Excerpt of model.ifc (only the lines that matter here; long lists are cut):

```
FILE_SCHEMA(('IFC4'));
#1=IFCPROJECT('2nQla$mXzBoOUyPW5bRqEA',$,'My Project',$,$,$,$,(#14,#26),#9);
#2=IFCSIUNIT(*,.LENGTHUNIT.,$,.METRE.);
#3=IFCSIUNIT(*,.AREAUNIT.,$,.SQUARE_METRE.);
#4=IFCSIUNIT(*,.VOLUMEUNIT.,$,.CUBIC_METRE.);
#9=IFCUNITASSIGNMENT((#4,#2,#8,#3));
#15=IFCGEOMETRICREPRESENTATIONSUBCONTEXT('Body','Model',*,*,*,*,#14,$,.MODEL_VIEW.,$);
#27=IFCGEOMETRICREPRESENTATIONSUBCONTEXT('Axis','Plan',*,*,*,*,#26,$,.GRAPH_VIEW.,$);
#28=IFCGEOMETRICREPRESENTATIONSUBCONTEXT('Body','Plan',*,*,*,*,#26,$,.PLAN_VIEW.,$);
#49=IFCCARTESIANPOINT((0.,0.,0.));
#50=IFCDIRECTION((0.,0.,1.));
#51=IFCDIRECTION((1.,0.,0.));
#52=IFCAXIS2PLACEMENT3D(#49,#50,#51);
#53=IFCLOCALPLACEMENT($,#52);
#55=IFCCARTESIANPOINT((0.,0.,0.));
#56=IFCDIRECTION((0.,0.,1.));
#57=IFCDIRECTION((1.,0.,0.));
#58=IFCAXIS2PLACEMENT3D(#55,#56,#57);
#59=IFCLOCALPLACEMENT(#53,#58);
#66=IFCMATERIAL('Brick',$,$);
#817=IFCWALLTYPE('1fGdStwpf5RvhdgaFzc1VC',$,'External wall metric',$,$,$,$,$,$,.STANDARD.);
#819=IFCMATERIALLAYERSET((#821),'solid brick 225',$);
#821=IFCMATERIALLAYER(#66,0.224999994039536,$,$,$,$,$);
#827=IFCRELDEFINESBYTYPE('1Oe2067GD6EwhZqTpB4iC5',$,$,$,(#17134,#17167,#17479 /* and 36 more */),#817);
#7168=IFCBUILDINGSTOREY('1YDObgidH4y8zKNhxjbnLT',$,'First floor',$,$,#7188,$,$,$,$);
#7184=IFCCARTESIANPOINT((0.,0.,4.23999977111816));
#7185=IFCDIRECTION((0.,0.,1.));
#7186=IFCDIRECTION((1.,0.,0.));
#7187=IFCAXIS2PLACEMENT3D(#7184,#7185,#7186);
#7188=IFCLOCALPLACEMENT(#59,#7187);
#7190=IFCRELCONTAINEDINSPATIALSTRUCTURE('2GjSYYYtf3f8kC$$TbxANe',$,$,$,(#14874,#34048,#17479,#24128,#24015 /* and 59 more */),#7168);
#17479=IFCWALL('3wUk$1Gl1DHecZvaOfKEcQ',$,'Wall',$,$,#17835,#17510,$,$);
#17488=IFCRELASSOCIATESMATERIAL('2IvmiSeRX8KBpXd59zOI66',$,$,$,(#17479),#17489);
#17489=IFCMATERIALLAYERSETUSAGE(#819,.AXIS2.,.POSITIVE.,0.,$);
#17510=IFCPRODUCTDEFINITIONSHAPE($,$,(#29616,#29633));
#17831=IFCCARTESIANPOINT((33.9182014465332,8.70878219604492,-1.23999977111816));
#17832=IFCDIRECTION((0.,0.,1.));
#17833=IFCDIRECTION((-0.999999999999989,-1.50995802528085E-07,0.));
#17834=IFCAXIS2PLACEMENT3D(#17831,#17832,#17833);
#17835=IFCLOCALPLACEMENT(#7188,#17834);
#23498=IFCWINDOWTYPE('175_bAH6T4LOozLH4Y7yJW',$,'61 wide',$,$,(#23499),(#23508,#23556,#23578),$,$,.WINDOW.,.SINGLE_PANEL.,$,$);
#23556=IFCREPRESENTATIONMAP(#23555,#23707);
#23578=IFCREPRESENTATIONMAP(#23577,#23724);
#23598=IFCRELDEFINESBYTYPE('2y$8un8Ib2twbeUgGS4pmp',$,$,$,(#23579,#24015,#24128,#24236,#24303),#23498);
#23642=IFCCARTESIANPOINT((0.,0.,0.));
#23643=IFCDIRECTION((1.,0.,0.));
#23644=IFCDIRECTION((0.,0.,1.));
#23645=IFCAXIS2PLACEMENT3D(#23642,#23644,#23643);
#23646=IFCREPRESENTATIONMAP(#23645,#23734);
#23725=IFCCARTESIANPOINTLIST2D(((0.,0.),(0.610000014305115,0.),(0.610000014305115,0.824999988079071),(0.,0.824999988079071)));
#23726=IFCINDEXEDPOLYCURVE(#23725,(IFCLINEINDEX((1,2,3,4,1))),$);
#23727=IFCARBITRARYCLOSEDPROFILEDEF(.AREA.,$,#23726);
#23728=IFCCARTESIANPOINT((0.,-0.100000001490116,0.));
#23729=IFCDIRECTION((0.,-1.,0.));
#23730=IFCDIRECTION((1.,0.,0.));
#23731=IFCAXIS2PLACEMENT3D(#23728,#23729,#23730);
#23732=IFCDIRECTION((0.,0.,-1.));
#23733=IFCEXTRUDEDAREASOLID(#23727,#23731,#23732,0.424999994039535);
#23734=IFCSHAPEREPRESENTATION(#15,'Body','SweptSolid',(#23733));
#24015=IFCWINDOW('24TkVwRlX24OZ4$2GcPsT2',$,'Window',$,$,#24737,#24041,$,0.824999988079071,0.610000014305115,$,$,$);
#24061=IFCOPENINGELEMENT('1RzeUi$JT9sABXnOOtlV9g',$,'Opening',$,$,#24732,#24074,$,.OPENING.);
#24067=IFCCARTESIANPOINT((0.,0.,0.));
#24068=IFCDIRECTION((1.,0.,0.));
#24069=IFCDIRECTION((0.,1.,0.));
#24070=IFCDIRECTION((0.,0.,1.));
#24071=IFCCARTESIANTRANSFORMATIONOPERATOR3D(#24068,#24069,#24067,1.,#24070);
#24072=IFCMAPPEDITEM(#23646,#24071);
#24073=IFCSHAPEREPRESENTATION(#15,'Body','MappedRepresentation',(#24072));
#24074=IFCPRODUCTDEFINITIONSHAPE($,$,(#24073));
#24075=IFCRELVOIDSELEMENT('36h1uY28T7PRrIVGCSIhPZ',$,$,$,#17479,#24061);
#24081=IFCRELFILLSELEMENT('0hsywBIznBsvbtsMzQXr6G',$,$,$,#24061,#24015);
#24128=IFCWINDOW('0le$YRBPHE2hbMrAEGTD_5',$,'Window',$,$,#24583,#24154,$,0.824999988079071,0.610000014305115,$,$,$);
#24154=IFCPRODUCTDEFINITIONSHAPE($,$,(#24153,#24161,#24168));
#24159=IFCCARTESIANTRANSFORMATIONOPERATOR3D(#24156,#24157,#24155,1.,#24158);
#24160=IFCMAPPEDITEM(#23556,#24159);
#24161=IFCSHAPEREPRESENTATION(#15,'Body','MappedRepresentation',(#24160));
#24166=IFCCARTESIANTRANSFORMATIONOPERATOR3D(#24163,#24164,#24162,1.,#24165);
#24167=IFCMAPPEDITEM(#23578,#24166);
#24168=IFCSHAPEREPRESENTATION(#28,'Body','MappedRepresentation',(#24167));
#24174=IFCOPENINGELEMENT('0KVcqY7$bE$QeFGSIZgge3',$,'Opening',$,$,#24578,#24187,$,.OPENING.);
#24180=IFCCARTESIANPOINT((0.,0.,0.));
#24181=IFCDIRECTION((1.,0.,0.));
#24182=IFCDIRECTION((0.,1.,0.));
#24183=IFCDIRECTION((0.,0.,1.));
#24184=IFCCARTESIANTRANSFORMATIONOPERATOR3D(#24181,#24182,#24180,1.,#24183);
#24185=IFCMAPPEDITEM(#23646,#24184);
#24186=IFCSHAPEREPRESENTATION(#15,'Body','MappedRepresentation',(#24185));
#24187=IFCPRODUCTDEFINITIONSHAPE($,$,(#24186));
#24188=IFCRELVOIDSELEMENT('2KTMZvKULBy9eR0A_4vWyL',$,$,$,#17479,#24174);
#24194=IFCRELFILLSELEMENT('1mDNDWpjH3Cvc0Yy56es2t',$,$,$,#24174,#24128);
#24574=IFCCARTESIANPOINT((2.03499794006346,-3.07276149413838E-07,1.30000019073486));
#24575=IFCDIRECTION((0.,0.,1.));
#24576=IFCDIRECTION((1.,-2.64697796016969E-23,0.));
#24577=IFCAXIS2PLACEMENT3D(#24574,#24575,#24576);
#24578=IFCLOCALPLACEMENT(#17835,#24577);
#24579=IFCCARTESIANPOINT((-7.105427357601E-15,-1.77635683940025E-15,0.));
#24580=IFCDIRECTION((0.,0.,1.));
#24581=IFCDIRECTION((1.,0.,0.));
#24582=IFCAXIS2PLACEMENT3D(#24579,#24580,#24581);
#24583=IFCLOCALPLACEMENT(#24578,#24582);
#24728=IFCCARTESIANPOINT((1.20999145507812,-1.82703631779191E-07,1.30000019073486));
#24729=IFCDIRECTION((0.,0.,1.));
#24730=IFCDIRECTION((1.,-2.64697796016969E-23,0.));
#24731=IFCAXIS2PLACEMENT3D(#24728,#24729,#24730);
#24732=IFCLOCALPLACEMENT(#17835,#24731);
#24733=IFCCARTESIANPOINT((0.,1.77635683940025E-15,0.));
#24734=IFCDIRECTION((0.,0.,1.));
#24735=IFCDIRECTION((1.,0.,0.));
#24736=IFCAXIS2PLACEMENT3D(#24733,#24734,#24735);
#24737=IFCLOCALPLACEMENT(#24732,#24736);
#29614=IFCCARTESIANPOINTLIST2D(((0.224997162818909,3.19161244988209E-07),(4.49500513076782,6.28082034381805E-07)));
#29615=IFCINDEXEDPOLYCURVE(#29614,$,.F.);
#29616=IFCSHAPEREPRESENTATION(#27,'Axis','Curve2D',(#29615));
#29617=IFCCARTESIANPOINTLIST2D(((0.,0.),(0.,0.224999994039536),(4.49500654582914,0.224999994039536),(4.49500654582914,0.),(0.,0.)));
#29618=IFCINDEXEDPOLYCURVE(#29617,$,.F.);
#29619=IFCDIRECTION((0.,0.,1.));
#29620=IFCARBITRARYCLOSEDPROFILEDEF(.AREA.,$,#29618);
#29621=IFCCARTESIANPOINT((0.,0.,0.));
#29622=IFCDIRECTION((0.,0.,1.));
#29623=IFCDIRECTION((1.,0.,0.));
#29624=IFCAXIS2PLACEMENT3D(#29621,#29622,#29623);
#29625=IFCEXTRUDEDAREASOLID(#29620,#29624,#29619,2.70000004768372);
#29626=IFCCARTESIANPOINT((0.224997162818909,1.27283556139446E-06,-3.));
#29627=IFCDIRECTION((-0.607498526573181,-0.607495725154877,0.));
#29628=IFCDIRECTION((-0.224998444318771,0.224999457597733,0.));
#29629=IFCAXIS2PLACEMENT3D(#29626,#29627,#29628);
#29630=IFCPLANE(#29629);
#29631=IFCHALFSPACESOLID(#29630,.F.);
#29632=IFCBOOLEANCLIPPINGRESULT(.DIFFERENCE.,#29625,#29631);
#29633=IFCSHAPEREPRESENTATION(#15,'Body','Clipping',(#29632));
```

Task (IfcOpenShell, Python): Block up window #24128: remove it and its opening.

```python
import ifcopenshell
import ifcopenshell.api.feature
import ifcopenshell.api.root
import ifcopenshell.geom
import ifcopenshell.util.shape

model = ifcopenshell.open("model.ifc")
settings = ifcopenshell.geom.settings()


def volume(element):
    """Net volume in cubic metres, openings subtracted."""
    shape = ifcopenshell.geom.create_shape(settings, element)
    return ifcopenshell.util.shape.get_volume(shape.geometry)


window = model.by_guid("0le$YRBPHE2hbMrAEGTD_5")
opening = window.FillsVoids[0].RelatingOpeningElement
wall = opening.VoidsElements[0].RelatingBuildingElement
before = volume(wall)

ifcopenshell.api.root.remove_product(model, product=window)
ifcopenshell.api.feature.remove_feature(model, feature=opening)

after = volume(wall)

print(f"wall volume {before:.3f} -> {after:.3f} m3")

model.write("model_edited.ifc")
```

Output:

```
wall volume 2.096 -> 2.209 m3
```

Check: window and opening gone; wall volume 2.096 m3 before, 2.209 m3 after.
